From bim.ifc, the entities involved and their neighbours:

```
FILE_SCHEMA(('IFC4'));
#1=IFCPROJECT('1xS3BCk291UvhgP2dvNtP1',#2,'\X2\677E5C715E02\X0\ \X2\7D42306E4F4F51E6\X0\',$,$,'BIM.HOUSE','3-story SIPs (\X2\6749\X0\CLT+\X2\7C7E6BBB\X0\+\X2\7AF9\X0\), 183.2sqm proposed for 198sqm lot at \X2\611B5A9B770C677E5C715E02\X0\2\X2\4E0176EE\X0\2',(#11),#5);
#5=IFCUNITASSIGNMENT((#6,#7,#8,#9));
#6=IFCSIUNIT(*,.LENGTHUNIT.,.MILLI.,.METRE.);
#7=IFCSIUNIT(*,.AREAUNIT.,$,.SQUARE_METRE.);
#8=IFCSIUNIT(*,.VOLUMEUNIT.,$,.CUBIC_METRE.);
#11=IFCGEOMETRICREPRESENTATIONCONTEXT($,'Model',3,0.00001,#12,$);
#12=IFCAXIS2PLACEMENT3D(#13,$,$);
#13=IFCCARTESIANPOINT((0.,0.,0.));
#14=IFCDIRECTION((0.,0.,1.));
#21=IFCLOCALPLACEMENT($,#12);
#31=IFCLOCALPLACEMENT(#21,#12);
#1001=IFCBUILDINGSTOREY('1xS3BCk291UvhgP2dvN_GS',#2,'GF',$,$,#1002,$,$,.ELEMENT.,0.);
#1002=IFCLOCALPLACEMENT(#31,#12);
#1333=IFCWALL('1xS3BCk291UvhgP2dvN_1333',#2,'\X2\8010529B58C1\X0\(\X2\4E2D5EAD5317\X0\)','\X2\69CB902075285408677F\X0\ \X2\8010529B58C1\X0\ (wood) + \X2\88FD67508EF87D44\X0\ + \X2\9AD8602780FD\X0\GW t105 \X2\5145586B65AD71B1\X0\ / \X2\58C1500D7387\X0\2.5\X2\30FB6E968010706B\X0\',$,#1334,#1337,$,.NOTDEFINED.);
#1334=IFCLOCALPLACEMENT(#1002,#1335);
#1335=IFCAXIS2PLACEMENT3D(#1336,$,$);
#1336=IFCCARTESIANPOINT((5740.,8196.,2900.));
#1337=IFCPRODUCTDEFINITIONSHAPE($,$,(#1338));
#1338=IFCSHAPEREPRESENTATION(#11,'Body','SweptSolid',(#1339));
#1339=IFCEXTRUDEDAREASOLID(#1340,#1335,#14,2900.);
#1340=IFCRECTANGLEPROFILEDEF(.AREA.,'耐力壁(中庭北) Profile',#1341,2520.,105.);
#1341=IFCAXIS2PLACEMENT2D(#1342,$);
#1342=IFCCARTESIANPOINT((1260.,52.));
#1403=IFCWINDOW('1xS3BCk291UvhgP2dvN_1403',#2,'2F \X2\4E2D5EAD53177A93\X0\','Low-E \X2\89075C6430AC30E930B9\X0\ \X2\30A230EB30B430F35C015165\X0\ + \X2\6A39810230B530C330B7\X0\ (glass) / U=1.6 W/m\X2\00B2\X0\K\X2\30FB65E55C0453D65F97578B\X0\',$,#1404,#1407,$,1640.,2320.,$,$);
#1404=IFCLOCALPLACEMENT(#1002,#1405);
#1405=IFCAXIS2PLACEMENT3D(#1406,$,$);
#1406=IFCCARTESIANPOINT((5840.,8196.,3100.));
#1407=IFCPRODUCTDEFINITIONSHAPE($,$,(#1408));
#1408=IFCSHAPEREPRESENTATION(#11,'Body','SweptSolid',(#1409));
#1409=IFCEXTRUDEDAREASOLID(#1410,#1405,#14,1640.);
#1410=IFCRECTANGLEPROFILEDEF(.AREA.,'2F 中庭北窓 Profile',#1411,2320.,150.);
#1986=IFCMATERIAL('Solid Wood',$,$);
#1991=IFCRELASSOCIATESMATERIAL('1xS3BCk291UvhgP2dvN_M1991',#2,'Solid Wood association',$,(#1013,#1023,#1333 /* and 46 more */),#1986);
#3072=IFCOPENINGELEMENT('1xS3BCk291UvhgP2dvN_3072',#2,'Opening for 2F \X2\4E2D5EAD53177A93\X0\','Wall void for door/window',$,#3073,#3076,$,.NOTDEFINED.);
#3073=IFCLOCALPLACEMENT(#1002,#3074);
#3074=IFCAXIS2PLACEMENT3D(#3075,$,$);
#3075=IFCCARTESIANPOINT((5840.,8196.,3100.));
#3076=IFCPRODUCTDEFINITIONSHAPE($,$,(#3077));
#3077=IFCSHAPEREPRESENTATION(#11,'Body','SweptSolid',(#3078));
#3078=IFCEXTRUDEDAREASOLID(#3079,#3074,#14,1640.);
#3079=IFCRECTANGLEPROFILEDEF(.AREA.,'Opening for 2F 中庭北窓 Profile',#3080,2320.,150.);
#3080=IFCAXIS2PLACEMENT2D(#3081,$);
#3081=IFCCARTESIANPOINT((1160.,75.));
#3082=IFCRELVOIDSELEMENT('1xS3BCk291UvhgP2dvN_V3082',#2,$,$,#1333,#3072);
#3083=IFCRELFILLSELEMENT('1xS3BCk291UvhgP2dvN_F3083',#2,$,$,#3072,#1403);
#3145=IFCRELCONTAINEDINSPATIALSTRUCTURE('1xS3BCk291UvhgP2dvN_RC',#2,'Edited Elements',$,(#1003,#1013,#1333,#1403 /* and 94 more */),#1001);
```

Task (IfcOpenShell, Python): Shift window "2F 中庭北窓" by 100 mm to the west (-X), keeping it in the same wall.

```python
import ifcopenshell
import ifcopenshell.api.geometry
import ifcopenshell.util.placement

model = ifcopenshell.open("bim.ifc")

window = model.by_guid("1xS3BCk291UvhgP2dvN_1403")
opening = window.FillsVoids[0].RelatingOpeningElement
wall = opening.VoidsElements[0].RelatingBuildingElement

wall_matrix = ifcopenshell.util.placement.get_local_placement(wall.ObjectPlacement)
shift = wall_matrix[:3, 0] * -100.0
before = ifcopenshell.util.placement.get_local_placement(window.ObjectPlacement)[:3, 3].copy()

# The window is not placed relative to its opening, so move both.
for product in (opening, window):
    matrix = ifcopenshell.util.placement.get_local_placement(product.ObjectPlacement)
    matrix[:3, 3] += shift
    ifcopenshell.api.geometry.edit_object_placement(model, product=product, matrix=matrix, is_si=False)

after = ifcopenshell.util.placement.get_local_placement(window.ObjectPlacement)[:3, 3]
print("window moved by", (after - before).round(3) + 0.0)

model.write("bim_rev.ifc")
```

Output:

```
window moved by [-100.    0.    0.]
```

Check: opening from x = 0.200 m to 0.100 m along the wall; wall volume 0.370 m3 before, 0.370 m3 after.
